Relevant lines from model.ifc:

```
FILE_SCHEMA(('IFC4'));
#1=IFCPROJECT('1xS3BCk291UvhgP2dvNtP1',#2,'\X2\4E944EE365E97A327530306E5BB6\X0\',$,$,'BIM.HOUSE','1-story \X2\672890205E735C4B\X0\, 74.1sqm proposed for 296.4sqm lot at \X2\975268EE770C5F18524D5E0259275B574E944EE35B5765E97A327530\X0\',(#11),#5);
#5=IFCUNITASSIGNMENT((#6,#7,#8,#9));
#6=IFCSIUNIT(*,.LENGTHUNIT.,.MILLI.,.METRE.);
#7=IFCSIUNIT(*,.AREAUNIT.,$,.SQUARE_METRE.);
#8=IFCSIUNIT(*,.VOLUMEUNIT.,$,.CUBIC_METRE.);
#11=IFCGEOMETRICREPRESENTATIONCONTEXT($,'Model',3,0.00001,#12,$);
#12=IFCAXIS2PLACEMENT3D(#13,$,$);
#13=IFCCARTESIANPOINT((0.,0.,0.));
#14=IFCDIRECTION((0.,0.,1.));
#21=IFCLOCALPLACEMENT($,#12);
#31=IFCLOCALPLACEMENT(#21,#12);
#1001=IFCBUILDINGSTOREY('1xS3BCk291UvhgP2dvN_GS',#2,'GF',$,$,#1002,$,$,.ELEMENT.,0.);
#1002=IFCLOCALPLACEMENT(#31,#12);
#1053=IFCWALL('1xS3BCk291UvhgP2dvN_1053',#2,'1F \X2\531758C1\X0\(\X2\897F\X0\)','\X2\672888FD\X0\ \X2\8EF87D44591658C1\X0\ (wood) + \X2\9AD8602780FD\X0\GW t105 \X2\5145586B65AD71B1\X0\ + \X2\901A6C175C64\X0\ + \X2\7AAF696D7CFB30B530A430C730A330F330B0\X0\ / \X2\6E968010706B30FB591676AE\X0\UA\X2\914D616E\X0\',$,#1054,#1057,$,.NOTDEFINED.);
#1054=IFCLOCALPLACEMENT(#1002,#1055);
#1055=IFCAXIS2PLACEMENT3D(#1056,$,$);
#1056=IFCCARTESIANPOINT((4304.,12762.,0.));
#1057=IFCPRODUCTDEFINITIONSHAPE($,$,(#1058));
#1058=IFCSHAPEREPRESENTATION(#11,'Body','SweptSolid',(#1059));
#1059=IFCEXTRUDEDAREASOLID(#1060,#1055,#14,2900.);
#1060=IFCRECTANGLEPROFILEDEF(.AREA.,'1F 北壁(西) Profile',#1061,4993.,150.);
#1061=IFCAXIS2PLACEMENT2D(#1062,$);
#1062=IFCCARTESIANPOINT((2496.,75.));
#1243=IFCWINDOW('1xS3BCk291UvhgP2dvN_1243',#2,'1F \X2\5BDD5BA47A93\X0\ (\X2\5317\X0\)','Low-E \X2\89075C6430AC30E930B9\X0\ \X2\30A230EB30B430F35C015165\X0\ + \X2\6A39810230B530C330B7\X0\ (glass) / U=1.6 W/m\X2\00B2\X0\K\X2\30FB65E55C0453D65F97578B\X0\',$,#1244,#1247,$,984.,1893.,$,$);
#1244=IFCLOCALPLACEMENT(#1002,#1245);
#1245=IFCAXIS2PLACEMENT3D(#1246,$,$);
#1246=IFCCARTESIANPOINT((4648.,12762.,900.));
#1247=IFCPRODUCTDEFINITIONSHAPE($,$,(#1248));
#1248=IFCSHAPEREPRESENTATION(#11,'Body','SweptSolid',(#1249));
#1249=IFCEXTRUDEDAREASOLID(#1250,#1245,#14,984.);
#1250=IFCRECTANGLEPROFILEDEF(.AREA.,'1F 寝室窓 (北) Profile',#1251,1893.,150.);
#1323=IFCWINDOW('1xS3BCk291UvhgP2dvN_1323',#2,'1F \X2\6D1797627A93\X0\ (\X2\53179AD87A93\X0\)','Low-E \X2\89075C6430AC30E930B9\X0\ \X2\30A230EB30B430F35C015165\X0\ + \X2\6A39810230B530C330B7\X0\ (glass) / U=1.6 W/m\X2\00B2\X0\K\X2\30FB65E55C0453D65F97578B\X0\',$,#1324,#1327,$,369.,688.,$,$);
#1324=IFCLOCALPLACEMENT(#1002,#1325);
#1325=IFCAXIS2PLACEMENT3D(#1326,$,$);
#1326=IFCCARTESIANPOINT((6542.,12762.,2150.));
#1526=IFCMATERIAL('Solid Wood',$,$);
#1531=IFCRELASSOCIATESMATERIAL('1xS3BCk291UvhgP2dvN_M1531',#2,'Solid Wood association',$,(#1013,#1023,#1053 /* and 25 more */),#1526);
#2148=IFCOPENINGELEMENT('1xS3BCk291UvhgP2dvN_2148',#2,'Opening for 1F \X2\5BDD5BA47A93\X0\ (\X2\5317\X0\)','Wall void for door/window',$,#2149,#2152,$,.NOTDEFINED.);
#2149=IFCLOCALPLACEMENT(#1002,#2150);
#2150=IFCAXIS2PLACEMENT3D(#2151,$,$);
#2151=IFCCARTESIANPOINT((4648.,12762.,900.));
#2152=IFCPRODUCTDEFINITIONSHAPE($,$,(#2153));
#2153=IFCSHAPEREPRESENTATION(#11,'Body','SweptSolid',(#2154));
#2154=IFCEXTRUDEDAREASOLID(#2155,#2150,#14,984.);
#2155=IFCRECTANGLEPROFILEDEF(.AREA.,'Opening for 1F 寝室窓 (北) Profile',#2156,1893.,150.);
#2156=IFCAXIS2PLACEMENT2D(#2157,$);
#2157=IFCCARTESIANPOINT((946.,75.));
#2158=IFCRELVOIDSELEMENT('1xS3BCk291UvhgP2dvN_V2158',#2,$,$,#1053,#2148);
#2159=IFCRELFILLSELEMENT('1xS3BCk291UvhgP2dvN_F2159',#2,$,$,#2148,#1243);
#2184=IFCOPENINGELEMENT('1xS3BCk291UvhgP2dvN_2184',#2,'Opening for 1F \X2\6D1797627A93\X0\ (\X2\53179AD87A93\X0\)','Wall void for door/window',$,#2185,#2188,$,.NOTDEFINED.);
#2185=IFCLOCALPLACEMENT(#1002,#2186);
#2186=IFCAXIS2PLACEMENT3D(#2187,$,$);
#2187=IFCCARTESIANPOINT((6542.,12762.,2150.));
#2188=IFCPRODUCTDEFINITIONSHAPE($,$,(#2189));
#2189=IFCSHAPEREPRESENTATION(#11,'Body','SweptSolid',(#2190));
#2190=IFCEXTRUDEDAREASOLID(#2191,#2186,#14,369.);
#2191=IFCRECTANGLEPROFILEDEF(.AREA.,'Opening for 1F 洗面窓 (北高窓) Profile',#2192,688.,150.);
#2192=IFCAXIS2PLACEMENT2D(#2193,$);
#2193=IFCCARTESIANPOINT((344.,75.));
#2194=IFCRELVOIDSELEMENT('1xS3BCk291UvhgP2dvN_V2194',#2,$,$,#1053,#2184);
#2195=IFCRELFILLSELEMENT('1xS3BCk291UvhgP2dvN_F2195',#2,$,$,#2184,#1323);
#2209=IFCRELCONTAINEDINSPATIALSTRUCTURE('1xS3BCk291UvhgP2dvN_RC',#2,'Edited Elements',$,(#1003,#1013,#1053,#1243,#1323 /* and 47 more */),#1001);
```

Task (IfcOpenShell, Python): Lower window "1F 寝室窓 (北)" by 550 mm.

```python
import numpy as np
import ifcopenshell
import ifcopenshell.api.geometry
import ifcopenshell.util.placement
import ifcopenshell.util.unit

model = ifcopenshell.open("model.ifc")
unit_scale = ifcopenshell.util.unit.calculate_unit_scale(model)

window = model.by_guid("1xS3BCk291UvhgP2dvN_1243")
opening = window.FillsVoids[0].RelatingOpeningElement
dz = -0.55 / unit_scale

shift = np.array([0.0, 0.0, dz])
# The window is not placed relative to its opening, so move both.
for product in (opening, window):
    matrix = ifcopenshell.util.placement.get_local_placement(product.ObjectPlacement)
    matrix[:3, 3] += shift
    ifcopenshell.api.geometry.edit_object_placement(model, product=product, matrix=matrix, is_si=False)

print(f"moved by {dz * unit_scale:+.3f} m")

model.write("model_updated.ifc")
```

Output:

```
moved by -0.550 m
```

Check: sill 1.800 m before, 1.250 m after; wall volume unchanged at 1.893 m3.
